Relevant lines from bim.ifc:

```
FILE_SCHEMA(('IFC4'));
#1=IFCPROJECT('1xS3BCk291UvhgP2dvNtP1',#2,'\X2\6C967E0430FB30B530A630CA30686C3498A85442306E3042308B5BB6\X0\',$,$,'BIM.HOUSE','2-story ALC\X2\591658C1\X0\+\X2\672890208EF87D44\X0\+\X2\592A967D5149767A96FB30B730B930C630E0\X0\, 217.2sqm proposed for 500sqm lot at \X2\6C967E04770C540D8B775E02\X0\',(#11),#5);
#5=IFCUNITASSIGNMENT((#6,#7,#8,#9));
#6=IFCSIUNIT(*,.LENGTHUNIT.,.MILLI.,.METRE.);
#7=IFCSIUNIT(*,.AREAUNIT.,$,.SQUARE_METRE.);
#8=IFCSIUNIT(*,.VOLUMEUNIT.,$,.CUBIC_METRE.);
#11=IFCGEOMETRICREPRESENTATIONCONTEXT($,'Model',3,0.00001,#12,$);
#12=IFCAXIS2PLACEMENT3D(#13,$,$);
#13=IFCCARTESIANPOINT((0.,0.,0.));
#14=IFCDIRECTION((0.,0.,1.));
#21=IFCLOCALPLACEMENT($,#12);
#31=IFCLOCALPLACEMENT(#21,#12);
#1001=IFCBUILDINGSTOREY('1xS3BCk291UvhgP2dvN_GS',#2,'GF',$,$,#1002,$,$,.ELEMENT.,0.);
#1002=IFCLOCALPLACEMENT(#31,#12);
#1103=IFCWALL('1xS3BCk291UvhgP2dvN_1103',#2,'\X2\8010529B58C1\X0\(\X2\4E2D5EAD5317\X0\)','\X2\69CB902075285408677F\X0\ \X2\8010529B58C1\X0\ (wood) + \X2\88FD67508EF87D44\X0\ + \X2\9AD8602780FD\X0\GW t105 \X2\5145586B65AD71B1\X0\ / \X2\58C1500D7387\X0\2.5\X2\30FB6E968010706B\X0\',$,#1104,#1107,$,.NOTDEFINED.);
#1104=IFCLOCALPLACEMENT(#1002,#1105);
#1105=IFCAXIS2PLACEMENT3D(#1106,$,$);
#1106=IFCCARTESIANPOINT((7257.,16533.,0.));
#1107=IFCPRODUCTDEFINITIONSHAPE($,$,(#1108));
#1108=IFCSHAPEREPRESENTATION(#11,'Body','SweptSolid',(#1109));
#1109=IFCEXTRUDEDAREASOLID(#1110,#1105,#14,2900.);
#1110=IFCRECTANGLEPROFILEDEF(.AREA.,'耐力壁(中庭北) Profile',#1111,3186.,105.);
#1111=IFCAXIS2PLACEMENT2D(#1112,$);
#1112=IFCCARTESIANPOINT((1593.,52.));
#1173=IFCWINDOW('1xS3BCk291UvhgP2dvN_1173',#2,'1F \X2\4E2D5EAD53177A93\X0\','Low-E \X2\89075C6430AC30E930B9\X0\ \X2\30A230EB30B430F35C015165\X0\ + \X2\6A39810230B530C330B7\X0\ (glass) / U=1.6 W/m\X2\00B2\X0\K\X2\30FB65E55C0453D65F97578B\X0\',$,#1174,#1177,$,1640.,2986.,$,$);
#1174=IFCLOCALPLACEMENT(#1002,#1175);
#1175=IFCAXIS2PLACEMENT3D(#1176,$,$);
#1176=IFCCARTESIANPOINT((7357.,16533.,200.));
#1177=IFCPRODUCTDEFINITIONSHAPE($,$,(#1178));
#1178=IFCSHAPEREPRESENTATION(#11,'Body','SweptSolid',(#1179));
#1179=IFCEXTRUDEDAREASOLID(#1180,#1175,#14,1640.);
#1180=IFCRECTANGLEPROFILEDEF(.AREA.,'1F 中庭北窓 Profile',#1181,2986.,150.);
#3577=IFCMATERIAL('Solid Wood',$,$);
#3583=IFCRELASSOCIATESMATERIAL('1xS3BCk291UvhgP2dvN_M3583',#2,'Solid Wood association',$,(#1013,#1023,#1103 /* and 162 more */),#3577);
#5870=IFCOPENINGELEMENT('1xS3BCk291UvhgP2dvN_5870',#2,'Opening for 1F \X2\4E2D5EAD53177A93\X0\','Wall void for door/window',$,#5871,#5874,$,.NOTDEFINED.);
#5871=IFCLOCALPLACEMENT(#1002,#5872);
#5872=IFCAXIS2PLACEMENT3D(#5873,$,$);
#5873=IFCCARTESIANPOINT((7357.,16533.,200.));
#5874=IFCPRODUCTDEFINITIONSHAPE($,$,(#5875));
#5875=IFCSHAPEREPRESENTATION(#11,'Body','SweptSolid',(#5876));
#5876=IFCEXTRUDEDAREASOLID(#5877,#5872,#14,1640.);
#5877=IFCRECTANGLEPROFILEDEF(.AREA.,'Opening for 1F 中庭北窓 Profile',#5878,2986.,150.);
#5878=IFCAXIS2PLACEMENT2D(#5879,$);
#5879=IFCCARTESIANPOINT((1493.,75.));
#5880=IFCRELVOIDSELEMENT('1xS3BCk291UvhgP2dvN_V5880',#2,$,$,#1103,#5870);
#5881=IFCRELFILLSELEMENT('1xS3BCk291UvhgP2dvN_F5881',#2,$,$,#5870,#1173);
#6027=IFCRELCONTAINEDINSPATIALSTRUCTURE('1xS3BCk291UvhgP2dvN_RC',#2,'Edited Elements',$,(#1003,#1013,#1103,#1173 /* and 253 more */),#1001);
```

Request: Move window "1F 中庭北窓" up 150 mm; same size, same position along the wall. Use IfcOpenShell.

```python
import numpy as np
import ifcopenshell
import ifcopenshell.api.geometry
import ifcopenshell.util.placement
import ifcopenshell.util.unit

model = ifcopenshell.open("bim.ifc")
unit_scale = ifcopenshell.util.unit.calculate_unit_scale(model)

window = model.by_guid("1xS3BCk291UvhgP2dvN_1173")
opening = window.FillsVoids[0].RelatingOpeningElement
dz = 150.0

shift = np.array([0.0, 0.0, dz])
# The window is not placed relative to its opening, so move both.
for product in (opening, window):
    matrix = ifcopenshell.util.placement.get_local_placement(product.ObjectPlacement)
    matrix[:3, 3] += shift
    ifcopenshell.api.geometry.edit_object_placement(model, product=product, matrix=matrix, is_si=False)

print(f"moved by {dz * unit_scale:+.3f} m")

model.write("bim_v2.ifc")
```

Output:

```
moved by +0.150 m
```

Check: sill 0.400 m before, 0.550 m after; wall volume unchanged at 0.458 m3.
